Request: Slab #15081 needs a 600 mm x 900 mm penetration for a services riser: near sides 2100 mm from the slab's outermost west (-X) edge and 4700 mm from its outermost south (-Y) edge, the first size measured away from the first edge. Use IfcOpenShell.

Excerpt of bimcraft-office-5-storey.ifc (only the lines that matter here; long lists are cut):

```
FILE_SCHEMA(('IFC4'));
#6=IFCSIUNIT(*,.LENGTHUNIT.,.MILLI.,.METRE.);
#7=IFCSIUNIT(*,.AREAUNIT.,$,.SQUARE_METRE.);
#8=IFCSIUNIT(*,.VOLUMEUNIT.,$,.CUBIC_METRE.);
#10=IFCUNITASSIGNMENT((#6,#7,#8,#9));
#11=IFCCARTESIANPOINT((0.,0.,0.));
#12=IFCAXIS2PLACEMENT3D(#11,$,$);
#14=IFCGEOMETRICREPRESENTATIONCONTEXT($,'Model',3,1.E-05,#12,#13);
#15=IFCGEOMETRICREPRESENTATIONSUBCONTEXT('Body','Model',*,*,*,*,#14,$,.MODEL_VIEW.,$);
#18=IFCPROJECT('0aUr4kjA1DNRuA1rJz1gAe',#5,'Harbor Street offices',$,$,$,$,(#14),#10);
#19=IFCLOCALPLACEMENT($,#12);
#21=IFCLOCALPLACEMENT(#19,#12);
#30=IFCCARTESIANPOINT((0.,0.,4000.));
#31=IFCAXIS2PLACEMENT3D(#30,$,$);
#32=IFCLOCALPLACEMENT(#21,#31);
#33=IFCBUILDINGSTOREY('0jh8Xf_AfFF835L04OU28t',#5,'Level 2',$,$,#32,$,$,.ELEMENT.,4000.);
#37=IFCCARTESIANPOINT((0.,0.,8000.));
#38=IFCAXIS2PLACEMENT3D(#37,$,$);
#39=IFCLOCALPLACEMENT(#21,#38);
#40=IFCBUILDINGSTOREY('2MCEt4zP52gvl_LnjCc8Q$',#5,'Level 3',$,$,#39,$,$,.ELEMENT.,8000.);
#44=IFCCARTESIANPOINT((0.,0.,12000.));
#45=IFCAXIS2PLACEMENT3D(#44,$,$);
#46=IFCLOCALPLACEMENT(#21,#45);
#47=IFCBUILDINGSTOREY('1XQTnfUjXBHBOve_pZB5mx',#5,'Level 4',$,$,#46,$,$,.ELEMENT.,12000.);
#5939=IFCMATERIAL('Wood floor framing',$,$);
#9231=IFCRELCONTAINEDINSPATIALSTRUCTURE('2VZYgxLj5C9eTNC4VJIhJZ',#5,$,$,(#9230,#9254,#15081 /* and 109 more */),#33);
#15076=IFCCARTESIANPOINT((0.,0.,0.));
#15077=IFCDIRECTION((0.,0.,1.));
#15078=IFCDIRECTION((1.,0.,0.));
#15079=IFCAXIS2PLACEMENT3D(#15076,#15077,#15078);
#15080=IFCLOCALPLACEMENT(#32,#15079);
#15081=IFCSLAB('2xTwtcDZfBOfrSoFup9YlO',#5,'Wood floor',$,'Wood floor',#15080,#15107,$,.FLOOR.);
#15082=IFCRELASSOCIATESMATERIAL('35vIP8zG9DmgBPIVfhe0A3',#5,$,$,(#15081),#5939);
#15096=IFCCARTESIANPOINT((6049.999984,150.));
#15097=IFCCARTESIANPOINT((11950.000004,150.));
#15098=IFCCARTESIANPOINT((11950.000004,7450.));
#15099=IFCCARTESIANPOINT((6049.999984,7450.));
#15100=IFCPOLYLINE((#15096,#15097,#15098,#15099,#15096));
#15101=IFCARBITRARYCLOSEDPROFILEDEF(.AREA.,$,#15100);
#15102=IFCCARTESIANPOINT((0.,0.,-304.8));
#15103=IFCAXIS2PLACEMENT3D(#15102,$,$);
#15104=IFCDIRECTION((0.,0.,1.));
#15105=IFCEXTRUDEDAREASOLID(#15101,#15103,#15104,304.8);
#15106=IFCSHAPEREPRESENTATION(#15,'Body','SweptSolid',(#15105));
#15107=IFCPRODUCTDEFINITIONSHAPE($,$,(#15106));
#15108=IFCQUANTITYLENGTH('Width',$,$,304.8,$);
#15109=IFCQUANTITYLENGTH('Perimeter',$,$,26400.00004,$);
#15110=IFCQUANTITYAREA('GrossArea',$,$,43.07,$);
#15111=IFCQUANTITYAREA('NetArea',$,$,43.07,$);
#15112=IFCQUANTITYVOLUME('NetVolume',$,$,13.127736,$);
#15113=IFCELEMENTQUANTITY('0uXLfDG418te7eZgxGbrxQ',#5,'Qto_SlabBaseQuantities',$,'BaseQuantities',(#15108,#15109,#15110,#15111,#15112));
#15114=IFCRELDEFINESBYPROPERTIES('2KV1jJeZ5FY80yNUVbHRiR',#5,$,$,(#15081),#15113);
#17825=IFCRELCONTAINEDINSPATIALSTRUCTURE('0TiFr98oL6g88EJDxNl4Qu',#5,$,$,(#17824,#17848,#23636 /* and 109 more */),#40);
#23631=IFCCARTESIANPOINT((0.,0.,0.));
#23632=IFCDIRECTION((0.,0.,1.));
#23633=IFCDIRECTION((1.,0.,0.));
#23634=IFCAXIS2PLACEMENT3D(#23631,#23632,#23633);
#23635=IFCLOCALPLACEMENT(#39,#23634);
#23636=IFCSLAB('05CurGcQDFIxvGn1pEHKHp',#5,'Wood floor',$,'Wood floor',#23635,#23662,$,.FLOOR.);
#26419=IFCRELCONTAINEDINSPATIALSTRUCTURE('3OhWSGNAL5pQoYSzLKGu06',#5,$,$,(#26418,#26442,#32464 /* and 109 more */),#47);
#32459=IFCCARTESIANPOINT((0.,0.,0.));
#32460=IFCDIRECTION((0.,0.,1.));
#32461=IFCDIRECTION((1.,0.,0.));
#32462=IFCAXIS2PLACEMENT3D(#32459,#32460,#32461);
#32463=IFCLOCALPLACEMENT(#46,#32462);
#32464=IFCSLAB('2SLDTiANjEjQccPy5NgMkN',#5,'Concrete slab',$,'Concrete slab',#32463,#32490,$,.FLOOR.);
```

```python
import numpy as np
import ifcopenshell
import ifcopenshell.api.feature
import ifcopenshell.api.geometry
import ifcopenshell.api.pset
import ifcopenshell.api.root
import ifcopenshell.geom
import ifcopenshell.util.element
import ifcopenshell.util.placement
import ifcopenshell.util.representation
import ifcopenshell.util.shape
import ifcopenshell.util.unit

model = ifcopenshell.open("bimcraft-office-5-storey.ifc")
unit_scale = ifcopenshell.util.unit.calculate_unit_scale(model)
area_scale = ifcopenshell.util.unit.calculate_unit_scale(model, "AREAUNIT")
volume_scale = ifcopenshell.util.unit.calculate_unit_scale(model, "VOLUMEUNIT")
settings = ifcopenshell.geom.settings()


def volume(element):
    """Net volume in cubic metres, openings subtracted."""
    shape = ifcopenshell.geom.create_shape(settings, element)
    return ifcopenshell.util.shape.get_volume(shape.geometry)


slab = model.by_id(15081)
before = volume(slab)

# Extent in the slab's own axes, in metres. The edges named are its -X and -Y sides.
slab_shape = ifcopenshell.geom.create_shape(settings, slab)
vertices = ifcopenshell.util.shape.get_vertices(slab_shape.geometry)
x_min, y_min, bottom = vertices.min(axis=0)
top = vertices[:, 2].max()

opening = ifcopenshell.api.root.create_entity(model, ifc_class="IfcOpeningElement", name="Services riser opening", predefined_type="OPENING")
context = ifcopenshell.util.representation.get_context(model, "Model", "Body", "MODEL_VIEW")
width, depth = 0.6, 0.9
outline = [(0.0, 0.0), (width, 0.0), (width, depth), (0.0, depth), (0.0, 0.0)]
# Overshoot both faces by 50 mm so the cut is clean.
shape = ifcopenshell.api.geometry.add_slab_representation(
    model, context=context, depth=top - bottom + 0.1, polyline=outline
)
ifcopenshell.api.geometry.assign_representation(model, product=opening, representation=shape)

matrix = ifcopenshell.util.placement.get_local_placement(slab.ObjectPlacement)
matrix[:, 3] = matrix @ np.append(np.array([x_min + 2.1, y_min + 4.7, bottom - 0.05]) / unit_scale, 1.0)
ifcopenshell.api.geometry.edit_object_placement(model, product=opening, matrix=matrix, is_si=False)
ifcopenshell.api.feature.add_feature(model, feature=opening, element=slab)

after = volume(slab)

# Update the slab's stored quantities.
qto = model.by_id(ifcopenshell.util.element.get_pset(slab, "Qto_SlabBaseQuantities", should_inherit=False)["id"])
ifcopenshell.api.pset.edit_qto(model, qto=qto, properties={
    "NetArea": after / (top - bottom) / area_scale,
    "NetVolume": after / volume_scale,
})

print(f"slab volume {before:.3f} -> {after:.3f} m3")

model.write("bimcraft-office-5-storey_updated.ifc")
```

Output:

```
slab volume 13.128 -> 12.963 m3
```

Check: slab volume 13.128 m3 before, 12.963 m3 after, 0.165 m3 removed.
